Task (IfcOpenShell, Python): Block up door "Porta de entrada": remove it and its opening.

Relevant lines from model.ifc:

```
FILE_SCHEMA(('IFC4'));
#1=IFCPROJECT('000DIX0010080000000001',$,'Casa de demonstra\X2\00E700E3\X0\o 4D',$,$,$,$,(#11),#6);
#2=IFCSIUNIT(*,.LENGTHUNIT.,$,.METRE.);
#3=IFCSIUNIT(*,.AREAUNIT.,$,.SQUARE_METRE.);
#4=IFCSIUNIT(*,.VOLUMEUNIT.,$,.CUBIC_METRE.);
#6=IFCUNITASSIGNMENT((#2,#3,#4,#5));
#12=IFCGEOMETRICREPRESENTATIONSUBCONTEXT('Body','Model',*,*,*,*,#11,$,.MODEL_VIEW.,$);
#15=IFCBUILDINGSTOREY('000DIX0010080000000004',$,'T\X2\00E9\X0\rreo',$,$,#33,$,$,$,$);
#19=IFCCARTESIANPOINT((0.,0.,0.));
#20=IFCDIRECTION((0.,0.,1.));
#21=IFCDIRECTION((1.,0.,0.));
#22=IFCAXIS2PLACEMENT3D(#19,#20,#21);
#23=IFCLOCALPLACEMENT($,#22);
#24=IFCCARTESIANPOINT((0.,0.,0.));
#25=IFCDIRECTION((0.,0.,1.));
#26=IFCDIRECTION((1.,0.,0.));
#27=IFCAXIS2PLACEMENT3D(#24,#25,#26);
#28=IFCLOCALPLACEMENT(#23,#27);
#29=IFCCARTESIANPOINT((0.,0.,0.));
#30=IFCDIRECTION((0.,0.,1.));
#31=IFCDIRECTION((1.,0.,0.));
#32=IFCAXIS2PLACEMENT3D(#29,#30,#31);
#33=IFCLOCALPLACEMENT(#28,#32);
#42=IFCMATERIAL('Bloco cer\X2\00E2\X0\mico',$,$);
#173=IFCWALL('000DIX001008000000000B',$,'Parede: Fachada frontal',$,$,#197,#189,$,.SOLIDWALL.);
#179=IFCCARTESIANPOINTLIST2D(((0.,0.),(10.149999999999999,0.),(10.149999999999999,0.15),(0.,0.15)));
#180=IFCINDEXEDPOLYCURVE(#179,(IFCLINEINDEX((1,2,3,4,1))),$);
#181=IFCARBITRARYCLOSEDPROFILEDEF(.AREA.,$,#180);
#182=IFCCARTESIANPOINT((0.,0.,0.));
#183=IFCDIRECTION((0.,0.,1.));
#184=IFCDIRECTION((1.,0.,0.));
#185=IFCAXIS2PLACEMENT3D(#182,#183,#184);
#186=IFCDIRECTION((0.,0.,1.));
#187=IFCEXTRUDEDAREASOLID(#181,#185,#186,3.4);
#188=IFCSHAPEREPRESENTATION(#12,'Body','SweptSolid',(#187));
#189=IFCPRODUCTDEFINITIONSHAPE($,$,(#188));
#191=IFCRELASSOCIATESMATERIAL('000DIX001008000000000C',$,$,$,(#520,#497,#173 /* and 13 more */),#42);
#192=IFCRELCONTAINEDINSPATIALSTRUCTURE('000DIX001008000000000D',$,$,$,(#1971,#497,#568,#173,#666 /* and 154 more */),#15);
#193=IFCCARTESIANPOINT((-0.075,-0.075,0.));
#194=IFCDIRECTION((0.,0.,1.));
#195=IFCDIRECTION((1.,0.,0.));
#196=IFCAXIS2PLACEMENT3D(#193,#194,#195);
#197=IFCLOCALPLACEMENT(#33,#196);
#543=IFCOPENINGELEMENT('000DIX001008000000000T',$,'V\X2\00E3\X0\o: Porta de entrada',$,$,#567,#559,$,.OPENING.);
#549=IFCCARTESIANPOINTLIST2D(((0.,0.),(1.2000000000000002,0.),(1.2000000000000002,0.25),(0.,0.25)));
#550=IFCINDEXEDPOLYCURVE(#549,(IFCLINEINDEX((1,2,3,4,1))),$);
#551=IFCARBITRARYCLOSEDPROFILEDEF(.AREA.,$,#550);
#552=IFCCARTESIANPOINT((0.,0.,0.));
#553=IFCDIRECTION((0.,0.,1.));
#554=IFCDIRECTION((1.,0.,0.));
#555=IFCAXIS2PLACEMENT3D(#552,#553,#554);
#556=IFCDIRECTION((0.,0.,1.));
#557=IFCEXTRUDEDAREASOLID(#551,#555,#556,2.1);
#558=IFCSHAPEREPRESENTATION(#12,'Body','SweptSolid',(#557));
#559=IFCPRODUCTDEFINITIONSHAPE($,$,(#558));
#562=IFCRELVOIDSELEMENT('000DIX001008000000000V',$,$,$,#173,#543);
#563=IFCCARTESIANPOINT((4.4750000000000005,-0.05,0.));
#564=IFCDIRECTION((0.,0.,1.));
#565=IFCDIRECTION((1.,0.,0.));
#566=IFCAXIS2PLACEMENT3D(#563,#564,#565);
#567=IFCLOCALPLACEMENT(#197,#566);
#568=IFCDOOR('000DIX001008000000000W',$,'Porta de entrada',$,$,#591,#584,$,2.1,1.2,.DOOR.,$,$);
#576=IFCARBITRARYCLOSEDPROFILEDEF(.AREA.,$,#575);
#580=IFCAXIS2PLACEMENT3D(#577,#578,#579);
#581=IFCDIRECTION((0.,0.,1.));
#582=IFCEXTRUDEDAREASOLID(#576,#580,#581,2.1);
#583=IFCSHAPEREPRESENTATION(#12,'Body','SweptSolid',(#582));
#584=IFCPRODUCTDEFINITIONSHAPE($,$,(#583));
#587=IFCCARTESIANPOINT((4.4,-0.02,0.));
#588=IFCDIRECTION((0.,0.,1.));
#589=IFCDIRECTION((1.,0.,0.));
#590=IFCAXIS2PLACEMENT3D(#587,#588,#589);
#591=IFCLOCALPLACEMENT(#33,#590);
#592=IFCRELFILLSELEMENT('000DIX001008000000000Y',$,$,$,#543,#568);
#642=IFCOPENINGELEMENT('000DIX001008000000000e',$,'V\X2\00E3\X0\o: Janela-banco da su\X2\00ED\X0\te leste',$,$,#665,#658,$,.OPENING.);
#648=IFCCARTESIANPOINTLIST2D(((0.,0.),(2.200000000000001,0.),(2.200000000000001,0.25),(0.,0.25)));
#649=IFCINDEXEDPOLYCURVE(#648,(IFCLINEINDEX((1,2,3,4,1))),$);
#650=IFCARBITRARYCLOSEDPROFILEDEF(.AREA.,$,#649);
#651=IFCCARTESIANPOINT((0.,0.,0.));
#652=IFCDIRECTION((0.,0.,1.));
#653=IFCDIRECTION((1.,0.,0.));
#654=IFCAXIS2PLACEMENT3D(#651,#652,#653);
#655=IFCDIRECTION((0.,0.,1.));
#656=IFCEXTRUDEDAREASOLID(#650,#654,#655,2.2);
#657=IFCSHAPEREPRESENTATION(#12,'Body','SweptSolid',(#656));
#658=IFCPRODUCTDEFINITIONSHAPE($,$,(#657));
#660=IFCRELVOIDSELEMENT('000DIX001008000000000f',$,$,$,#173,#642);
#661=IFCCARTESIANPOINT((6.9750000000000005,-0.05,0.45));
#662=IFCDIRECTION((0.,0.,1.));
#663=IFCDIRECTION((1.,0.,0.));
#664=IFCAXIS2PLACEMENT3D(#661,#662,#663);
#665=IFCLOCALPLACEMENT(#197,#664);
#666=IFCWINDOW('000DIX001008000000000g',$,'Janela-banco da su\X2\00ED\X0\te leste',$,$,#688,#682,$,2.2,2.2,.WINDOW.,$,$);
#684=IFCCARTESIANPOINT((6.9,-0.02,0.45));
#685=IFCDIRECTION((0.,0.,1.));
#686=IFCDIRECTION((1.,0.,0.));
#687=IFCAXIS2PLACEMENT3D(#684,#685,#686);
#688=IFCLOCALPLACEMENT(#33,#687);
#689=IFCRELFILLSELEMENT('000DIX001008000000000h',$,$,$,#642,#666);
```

```python
import ifcopenshell
import ifcopenshell.api.feature
import ifcopenshell.api.root
import ifcopenshell.geom
import ifcopenshell.util.shape

model = ifcopenshell.open("model.ifc")
settings = ifcopenshell.geom.settings()


def volume(element):
    """Net volume in cubic metres, openings subtracted."""
    shape = ifcopenshell.geom.create_shape(settings, element)
    return ifcopenshell.util.shape.get_volume(shape.geometry)


door = model.by_id(568)
opening = door.FillsVoids[0].RelatingOpeningElement
wall = opening.VoidsElements[0].RelatingBuildingElement
before = volume(wall)

ifcopenshell.api.root.remove_product(model, product=door)
ifcopenshell.api.feature.remove_feature(model, feature=opening)

after = volume(wall)

print(f"wall volume {before:.3f} -> {after:.3f} m3")

model.write("model_updated.ifc")
```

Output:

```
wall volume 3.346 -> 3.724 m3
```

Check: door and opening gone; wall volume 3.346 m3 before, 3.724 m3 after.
